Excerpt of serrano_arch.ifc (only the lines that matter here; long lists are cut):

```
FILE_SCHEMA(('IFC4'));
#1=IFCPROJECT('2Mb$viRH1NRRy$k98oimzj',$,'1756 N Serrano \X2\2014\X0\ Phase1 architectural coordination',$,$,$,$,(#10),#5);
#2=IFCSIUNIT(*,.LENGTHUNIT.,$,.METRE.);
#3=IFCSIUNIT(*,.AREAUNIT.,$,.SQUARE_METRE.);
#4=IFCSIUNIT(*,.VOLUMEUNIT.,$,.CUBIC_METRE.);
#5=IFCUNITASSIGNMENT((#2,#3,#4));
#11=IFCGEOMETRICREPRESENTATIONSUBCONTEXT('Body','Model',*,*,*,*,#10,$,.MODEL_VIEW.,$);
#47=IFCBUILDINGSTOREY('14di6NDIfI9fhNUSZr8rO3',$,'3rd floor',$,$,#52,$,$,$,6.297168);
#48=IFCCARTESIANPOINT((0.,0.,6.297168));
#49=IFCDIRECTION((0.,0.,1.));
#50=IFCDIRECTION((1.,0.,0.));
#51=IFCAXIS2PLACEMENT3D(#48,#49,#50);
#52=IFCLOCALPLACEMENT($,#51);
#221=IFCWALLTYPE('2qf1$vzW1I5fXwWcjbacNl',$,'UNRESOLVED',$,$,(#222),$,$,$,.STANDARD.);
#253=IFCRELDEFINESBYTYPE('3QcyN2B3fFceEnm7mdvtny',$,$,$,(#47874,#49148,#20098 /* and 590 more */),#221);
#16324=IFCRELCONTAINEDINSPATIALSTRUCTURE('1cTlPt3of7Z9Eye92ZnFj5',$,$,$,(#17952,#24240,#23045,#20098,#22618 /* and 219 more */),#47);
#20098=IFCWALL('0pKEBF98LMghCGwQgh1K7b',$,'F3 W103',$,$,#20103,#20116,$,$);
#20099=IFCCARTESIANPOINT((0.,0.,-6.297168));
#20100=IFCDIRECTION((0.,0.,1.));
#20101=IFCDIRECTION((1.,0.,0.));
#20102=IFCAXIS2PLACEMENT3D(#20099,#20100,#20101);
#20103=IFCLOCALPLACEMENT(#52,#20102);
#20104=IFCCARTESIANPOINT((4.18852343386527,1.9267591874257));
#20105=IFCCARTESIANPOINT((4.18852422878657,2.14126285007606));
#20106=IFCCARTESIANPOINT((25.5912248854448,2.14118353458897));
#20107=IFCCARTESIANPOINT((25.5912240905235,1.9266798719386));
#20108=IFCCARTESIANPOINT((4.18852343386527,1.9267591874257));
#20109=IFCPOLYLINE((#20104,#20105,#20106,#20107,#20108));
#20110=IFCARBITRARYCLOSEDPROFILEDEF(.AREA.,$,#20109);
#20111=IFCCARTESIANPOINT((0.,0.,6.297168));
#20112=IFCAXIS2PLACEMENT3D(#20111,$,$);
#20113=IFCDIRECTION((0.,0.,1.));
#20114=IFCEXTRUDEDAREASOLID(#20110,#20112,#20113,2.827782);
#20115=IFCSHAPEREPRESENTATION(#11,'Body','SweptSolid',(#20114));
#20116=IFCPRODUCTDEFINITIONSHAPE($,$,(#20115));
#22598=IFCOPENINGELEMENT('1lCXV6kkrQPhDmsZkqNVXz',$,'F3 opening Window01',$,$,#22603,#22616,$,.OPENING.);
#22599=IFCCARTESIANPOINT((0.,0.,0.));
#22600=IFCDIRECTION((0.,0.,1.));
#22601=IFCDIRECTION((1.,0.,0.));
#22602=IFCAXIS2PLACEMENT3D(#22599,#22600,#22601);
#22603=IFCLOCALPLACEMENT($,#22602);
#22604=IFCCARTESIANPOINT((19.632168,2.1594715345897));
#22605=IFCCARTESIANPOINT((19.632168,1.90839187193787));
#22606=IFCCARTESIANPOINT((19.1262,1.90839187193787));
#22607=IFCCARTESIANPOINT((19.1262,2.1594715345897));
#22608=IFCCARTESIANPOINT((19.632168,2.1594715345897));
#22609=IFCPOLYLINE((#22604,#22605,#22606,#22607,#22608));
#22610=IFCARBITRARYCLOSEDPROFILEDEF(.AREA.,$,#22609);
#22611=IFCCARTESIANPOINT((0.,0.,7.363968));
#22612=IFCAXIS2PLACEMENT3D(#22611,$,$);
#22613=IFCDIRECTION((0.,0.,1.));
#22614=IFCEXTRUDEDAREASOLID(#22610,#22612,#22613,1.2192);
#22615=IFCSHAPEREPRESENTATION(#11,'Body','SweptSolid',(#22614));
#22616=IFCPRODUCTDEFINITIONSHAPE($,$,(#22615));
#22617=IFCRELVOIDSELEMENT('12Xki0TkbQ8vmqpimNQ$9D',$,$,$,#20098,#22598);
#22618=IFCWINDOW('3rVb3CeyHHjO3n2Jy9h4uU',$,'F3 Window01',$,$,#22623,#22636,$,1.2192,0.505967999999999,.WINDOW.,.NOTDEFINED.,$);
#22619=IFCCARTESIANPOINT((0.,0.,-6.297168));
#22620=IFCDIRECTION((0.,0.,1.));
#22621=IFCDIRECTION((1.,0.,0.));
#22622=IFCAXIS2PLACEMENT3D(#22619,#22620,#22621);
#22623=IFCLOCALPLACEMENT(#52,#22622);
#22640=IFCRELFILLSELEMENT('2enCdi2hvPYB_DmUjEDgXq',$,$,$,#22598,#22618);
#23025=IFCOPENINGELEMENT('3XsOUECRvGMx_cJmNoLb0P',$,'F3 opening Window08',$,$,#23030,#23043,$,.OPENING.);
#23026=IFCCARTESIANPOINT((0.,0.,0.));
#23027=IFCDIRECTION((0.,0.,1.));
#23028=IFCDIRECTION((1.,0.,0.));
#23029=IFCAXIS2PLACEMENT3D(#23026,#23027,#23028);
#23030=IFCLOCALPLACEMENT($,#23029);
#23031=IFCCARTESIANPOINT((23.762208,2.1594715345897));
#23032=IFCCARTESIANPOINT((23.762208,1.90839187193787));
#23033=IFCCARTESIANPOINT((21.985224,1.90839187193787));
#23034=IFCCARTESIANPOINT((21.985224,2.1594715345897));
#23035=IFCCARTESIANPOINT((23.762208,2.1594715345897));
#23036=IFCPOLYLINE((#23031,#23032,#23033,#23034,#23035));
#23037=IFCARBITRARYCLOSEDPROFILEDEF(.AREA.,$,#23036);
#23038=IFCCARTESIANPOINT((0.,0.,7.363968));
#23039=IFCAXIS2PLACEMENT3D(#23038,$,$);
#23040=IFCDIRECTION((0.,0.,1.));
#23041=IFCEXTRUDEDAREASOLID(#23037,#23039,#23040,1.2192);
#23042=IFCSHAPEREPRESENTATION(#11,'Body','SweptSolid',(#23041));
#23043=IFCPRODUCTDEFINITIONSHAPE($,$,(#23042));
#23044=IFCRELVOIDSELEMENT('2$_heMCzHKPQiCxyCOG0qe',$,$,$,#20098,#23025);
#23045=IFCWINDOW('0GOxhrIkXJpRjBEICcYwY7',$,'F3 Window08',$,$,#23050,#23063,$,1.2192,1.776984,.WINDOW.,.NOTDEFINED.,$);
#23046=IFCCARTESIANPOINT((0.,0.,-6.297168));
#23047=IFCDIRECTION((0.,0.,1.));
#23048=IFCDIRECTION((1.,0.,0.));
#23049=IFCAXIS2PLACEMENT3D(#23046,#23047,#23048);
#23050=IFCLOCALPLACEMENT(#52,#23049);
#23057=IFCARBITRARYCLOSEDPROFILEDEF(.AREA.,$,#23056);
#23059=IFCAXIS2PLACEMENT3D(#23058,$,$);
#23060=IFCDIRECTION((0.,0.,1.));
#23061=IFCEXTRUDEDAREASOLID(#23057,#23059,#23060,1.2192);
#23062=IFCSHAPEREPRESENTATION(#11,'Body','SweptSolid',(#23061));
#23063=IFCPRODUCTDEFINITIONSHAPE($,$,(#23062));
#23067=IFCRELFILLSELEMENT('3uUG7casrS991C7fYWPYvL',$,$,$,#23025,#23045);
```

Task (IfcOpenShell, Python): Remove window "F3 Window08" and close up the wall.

```python
import ifcopenshell
import ifcopenshell.api.feature
import ifcopenshell.api.root
import ifcopenshell.geom
import ifcopenshell.util.shape

model = ifcopenshell.open("serrano_arch.ifc")
settings = ifcopenshell.geom.settings()


def volume(element):
    """Net volume in cubic metres, openings subtracted."""
    shape = ifcopenshell.geom.create_shape(settings, element)
    return ifcopenshell.util.shape.get_volume(shape.geometry)


window = model.by_guid("0GOxhrIkXJpRjBEICcYwY7")
opening = window.FillsVoids[0].RelatingOpeningElement
wall = opening.VoidsElements[0].RelatingBuildingElement
before = volume(wall)

ifcopenshell.api.root.remove_product(model, product=window)
ifcopenshell.api.feature.remove_feature(model, feature=opening)

after = volume(wall)

print(f"wall volume {before:.3f} -> {after:.3f} m3")

model.write("serrano_arch-out.ifc")
```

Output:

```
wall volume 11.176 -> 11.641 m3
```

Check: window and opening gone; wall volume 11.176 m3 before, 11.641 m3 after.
